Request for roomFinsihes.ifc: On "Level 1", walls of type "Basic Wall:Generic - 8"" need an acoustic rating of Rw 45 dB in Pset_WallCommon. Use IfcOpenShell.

First a look at what the model holds.

```python
import ifcopenshell
import ifcopenshell.util.element

model = ifcopenshell.open("roomFinsihes.ifc")
print(model.schema)
storey = next(s for s in model.by_type("IfcBuildingStorey") if s.Name == "Level 1")
walls = [e for e in ifcopenshell.util.element.get_decomposition(storey) if e.is_a("IfcWall")]
seen = {}
for e in walls:
    element_type = ifcopenshell.util.element.get_type(e)
    key = (element_type.Name if element_type != e and element_type else None, ifcopenshell.util.element.get_pset(e, "Pset_WallCommon", "AcousticRating"))
    seen[key] = seen.get(key, 0) + 1
for (name, value), count in sorted(seen.items(), key=str):
    print(count, "x", name, "|", value)
```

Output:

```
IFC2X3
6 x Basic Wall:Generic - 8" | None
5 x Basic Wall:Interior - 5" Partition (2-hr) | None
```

```python
import ifcopenshell
import ifcopenshell.api.pset
import ifcopenshell.util.element

model = ifcopenshell.open("roomFinsihes.ifc")

storey = next(s for s in model.by_type("IfcBuildingStorey") if s.Name == "Level 1")
walls = [e for e in ifcopenshell.util.element.get_decomposition(storey) if e.is_a("IfcWall")]

count = 0
for e in walls:
    element_type = ifcopenshell.util.element.get_type(e)
    if element_type in (None, e) or element_type.Name != 'Basic Wall:Generic - 8"':
        continue
    # add_pset returns the element's existing set when there is one.
    pset = ifcopenshell.api.pset.add_pset(model, product=e, name="Pset_WallCommon")
    ifcopenshell.api.pset.edit_pset(model, pset=pset, properties={"AcousticRating": "Rw 45 dB"})
    count += 1

print(count, "walls updated")

model.write("roomFinsihes_updated.ifc")
```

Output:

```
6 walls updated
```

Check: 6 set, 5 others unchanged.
